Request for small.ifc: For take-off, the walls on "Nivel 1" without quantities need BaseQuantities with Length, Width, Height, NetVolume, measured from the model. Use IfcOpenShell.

First a look at what the model holds.

```python
import ifcopenshell
import ifcopenshell.util.element
import ifcopenshell.util.unit

model = ifcopenshell.open("small.ifc")
print(model.schema)
for unit_type in ("LENGTHUNIT", "AREAUNIT", "VOLUMEUNIT"):
    print(unit_type, ifcopenshell.util.unit.calculate_unit_scale(model, unit_type))
storey = next(s for s in model.by_type("IfcBuildingStorey") if s.Name == "Nivel 1")
walls = [e for e in ifcopenshell.util.element.get_decomposition(storey) if e.is_a("IfcWall")]
for e in sorted(walls, key=lambda e: e.id()):
    print(e.id(), e.is_a(), e.Name, list(ifcopenshell.util.element.get_psets(e, qtos_only=True)), sep=" | ")
```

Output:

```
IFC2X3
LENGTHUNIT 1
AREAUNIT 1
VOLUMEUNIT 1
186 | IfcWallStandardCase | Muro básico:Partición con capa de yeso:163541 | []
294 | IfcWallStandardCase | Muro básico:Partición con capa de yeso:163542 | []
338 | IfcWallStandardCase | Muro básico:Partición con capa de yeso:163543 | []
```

```python
import ifcopenshell
import ifcopenshell.api.pset
import ifcopenshell.geom
import ifcopenshell.util.element
import ifcopenshell.util.shape
import ifcopenshell.util.unit

model = ifcopenshell.open("small.ifc")
unit_scale = ifcopenshell.util.unit.calculate_unit_scale(model)
volume_scale = ifcopenshell.util.unit.calculate_unit_scale(model, "VOLUMEUNIT")
settings = ifcopenshell.geom.settings()

storey = next(s for s in model.by_type("IfcBuildingStorey") if s.Name == "Nivel 1")
walls = [e for e in ifcopenshell.util.element.get_decomposition(storey) if e.is_a("IfcWall")]

for e in sorted(walls, key=lambda e: e.id()):
    if ifcopenshell.util.element.get_psets(e, qtos_only=True, should_inherit=False):
        continue
    # Geometry comes back in metres, in the element's own axes.
    shape = ifcopenshell.geom.create_shape(settings, e)
    values = {
        "Length": ifcopenshell.util.shape.get_x(shape.geometry) / unit_scale,
        "Width": ifcopenshell.util.shape.get_y(shape.geometry) / unit_scale,
        "Height": ifcopenshell.util.shape.get_z(shape.geometry) / unit_scale,
        "NetVolume": ifcopenshell.util.shape.get_volume(shape.geometry) / volume_scale,
    }
    qto = ifcopenshell.api.pset.add_qto(model, product=e, name="BaseQuantities")
    ifcopenshell.api.pset.edit_qto(model, qto=qto, properties=values)
    print(e.id(), {k: round(v, 3) for k, v in values.items()})

model.write("small_rev.ifc")
```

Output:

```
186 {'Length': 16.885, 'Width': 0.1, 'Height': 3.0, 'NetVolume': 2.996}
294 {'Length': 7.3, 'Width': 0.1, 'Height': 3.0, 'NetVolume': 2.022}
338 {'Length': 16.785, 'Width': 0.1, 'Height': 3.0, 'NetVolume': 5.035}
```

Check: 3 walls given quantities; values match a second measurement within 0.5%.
